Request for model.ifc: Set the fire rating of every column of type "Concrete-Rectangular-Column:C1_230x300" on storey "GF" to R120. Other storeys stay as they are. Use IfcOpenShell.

First a look at what the model holds.

```python
import ifcopenshell
import ifcopenshell.util.element

model = ifcopenshell.open("model.ifc")
print(model.schema)
storey = next(s for s in model.by_type("IfcBuildingStorey") if s.Name == "GF")
columns = [e for e in ifcopenshell.util.element.get_decomposition(storey) if e.is_a("IfcColumn")]
seen = {}
for e in columns:
    element_type = ifcopenshell.util.element.get_type(e)
    key = (element_type.Name if element_type != e and element_type else None, ifcopenshell.util.element.get_pset(e, "Pset_ColumnCommon", "FireRating"))
    seen[key] = seen.get(key, 0) + 1
for (name, value), count in sorted(seen.items(), key=str):
    print(count, "x", name, "|", value)
```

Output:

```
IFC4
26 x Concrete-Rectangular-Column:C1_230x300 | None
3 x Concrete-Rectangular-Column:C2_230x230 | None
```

```python
import ifcopenshell
import ifcopenshell.api.pset
import ifcopenshell.util.element

model = ifcopenshell.open("model.ifc")

storey = next(s for s in model.by_type("IfcBuildingStorey") if s.Name == "GF")
columns = [e for e in ifcopenshell.util.element.get_decomposition(storey) if e.is_a("IfcColumn")]

count = 0
for e in columns:
    element_type = ifcopenshell.util.element.get_type(e)
    if element_type in (None, e) or element_type.Name != "Concrete-Rectangular-Column:C1_230x300":
        continue
    # add_pset returns the element's existing set when there is one.
    pset = ifcopenshell.api.pset.add_pset(model, product=e, name="Pset_ColumnCommon")
    ifcopenshell.api.pset.edit_pset(model, pset=pset, properties={"FireRating": "R120"})
    count += 1

print(count, "columns updated")

model.write("model-out.ifc")
```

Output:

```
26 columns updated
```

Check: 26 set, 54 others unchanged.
